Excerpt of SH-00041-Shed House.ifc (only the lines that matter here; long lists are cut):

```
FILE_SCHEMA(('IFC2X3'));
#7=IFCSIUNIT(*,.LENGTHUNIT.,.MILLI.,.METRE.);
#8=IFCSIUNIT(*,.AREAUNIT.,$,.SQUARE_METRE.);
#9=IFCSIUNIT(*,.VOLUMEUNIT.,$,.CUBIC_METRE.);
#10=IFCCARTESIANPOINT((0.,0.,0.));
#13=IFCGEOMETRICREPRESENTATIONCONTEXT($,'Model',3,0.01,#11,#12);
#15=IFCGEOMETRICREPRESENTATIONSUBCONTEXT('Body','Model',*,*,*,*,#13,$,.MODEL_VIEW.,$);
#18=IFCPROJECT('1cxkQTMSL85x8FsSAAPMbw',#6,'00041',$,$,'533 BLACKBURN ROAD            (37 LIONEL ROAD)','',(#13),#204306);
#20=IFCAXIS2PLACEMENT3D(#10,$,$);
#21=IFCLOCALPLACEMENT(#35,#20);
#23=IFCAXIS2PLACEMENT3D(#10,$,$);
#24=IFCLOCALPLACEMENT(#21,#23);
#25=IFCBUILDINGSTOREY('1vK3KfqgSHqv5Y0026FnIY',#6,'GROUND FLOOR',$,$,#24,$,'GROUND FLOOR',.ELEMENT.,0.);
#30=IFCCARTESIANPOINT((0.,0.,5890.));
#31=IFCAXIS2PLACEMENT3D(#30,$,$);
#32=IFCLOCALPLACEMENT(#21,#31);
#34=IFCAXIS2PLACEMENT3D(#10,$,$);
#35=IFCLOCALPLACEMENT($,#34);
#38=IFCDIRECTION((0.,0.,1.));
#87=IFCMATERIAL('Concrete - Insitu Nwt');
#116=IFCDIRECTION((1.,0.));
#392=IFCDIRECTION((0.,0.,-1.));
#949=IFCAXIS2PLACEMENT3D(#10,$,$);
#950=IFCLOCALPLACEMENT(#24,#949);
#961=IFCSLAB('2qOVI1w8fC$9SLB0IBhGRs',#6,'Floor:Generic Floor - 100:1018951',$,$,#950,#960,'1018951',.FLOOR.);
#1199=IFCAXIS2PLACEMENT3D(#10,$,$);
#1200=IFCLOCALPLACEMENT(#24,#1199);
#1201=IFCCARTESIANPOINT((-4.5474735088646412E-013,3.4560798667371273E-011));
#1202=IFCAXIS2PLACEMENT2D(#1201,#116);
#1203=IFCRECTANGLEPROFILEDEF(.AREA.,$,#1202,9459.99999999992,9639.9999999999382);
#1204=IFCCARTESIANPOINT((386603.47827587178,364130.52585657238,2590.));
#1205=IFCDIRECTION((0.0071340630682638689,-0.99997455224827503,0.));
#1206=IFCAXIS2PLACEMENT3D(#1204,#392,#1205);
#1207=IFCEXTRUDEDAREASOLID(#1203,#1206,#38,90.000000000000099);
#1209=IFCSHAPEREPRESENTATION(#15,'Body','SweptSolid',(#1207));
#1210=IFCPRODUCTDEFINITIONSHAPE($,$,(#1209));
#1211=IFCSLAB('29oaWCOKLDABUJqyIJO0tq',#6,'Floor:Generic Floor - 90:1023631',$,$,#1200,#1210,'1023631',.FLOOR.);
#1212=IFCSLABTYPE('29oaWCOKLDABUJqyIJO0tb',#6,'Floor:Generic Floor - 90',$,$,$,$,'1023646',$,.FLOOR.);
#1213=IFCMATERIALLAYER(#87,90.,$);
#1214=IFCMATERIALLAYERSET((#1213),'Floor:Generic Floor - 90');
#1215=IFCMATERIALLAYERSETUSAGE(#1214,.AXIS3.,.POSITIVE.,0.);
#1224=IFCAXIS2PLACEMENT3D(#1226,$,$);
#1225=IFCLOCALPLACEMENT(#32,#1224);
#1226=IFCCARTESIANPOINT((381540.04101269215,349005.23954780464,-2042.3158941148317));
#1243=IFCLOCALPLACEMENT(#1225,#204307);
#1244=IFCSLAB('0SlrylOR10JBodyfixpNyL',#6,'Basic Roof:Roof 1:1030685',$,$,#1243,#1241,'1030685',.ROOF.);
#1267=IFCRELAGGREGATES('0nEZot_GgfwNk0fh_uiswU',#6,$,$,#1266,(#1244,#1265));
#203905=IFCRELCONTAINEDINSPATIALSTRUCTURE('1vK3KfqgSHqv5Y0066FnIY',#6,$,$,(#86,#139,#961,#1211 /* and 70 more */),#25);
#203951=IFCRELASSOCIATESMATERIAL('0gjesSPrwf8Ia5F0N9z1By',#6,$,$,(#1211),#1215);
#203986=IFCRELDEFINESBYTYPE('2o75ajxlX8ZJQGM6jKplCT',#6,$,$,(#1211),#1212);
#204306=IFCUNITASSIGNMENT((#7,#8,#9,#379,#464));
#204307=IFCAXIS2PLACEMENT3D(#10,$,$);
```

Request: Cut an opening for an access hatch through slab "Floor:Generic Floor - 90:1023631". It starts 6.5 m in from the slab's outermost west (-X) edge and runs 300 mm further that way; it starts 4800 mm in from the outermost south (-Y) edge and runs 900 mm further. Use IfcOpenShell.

```python
import numpy as np
import ifcopenshell
import ifcopenshell.api.feature
import ifcopenshell.api.geometry
import ifcopenshell.api.root
import ifcopenshell.geom
import ifcopenshell.util.placement
import ifcopenshell.util.representation
import ifcopenshell.util.shape
import ifcopenshell.util.unit

model = ifcopenshell.open("SH-00041-Shed House.ifc")
unit_scale = ifcopenshell.util.unit.calculate_unit_scale(model)
settings = ifcopenshell.geom.settings()


def volume(element):
    """Net volume in cubic metres, openings subtracted."""
    shape = ifcopenshell.geom.create_shape(settings, element)
    return ifcopenshell.util.shape.get_volume(shape.geometry)


slab = model.by_guid("29oaWCOKLDABUJqyIJO0tq")
before = volume(slab)

# Extent in the slab's own axes, in metres. The edges named are its -X and -Y sides.
slab_shape = ifcopenshell.geom.create_shape(settings, slab)
vertices = ifcopenshell.util.shape.get_vertices(slab_shape.geometry)
x_min, y_min, bottom = vertices.min(axis=0)
top = vertices[:, 2].max()

opening = ifcopenshell.api.root.create_entity(model, ifc_class="IfcOpeningElement", name="Access hatch opening")
context = ifcopenshell.util.representation.get_context(model, "Model", "Body", "MODEL_VIEW")
width, depth = 0.3, 0.9
outline = [(0.0, 0.0), (width, 0.0), (width, depth), (0.0, depth), (0.0, 0.0)]
# Overshoot both faces by 50 mm so the cut is clean.
shape = ifcopenshell.api.geometry.add_slab_representation(
    model, context=context, depth=top - bottom + 0.1, polyline=outline
)
ifcopenshell.api.geometry.assign_representation(model, product=opening, representation=shape)

matrix = ifcopenshell.util.placement.get_local_placement(slab.ObjectPlacement)
matrix[:, 3] = matrix @ np.append(np.array([x_min + 6.5, y_min + 4.8, bottom - 0.05]) / unit_scale, 1.0)
ifcopenshell.api.geometry.edit_object_placement(model, product=opening, matrix=matrix, is_si=False)
ifcopenshell.api.feature.add_feature(model, feature=opening, element=slab)

after = volume(slab)

print(f"slab volume {before:.3f} -> {after:.3f} m3")

model.write("SH-00041-Shed House_updated.ifc")
```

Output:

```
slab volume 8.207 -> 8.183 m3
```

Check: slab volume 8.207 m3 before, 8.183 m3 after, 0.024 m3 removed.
